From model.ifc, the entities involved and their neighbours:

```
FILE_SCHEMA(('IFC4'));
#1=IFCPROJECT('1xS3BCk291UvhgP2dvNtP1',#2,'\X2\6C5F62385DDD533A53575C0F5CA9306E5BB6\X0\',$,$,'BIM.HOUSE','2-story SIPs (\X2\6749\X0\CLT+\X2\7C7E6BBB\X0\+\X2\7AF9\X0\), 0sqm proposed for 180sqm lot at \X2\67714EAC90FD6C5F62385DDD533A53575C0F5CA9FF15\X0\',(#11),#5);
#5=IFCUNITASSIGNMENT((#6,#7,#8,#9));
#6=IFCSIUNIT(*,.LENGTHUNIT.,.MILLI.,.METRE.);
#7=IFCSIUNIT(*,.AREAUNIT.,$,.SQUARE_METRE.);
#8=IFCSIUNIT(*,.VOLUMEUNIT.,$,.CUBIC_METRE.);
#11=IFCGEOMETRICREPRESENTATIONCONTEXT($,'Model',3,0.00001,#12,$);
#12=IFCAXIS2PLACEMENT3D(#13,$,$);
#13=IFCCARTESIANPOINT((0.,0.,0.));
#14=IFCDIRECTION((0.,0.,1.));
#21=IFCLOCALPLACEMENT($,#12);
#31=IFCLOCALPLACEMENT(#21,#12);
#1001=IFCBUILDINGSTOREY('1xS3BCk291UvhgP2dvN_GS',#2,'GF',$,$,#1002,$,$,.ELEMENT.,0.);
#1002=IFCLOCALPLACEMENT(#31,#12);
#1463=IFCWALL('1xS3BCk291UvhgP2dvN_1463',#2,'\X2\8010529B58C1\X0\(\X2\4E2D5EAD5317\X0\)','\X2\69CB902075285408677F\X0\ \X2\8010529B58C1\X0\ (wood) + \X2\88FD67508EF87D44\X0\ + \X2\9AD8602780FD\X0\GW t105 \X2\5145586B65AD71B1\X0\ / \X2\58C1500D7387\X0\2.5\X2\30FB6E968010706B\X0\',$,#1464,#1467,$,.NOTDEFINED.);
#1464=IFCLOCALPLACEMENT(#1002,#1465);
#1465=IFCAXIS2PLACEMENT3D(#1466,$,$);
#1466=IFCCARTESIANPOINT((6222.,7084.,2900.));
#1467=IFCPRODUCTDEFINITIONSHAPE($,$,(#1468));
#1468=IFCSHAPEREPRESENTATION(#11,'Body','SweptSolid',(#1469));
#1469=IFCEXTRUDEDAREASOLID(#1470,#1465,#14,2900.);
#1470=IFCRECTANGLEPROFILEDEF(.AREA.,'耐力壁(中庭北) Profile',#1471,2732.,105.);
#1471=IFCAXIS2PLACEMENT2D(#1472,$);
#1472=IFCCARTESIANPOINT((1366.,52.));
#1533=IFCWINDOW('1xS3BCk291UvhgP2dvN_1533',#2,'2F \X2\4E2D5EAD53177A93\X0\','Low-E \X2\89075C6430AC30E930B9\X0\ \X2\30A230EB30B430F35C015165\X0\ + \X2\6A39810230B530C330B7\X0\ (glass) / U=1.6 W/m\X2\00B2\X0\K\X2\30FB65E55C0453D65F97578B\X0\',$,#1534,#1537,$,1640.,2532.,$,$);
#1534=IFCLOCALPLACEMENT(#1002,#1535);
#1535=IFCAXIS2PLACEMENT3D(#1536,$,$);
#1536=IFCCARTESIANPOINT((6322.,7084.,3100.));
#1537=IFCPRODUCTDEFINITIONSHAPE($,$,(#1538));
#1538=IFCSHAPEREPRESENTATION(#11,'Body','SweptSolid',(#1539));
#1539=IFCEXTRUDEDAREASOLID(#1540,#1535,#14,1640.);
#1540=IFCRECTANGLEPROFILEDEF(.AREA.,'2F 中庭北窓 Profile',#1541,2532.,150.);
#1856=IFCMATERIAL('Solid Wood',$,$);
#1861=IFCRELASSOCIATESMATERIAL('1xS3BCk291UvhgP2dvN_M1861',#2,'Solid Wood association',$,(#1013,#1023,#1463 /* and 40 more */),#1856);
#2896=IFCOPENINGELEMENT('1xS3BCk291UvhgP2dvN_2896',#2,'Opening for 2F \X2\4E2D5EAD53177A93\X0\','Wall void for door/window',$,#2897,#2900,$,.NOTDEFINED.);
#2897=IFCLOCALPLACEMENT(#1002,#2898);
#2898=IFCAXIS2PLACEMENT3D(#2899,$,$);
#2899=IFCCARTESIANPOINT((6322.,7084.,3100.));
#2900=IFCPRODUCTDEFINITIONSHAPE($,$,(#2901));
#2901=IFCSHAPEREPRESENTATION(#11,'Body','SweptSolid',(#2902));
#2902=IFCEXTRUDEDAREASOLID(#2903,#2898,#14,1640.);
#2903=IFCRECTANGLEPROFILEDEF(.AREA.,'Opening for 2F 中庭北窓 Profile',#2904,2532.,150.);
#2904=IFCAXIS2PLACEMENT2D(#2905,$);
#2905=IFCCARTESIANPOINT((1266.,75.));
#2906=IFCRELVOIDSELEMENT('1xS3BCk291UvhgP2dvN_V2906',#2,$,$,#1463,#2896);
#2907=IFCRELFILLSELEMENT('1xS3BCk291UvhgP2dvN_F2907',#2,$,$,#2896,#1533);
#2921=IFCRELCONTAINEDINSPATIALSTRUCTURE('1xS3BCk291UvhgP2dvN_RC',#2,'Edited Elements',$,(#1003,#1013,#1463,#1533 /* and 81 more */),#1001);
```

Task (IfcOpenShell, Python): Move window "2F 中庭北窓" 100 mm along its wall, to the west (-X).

```python
import ifcopenshell
import ifcopenshell.api.geometry
import ifcopenshell.util.placement

model = ifcopenshell.open("model.ifc")

window = model.by_id(1533)
opening = window.FillsVoids[0].RelatingOpeningElement
wall = opening.VoidsElements[0].RelatingBuildingElement

wall_matrix = ifcopenshell.util.placement.get_local_placement(wall.ObjectPlacement)
shift = wall_matrix[:3, 0] * -100.0
before = ifcopenshell.util.placement.get_local_placement(window.ObjectPlacement)[:3, 3].copy()

# The window is not placed relative to its opening, so move both.
for product in (opening, window):
    matrix = ifcopenshell.util.placement.get_local_placement(product.ObjectPlacement)
    matrix[:3, 3] += shift
    ifcopenshell.api.geometry.edit_object_placement(model, product=product, matrix=matrix, is_si=False)

after = ifcopenshell.util.placement.get_local_placement(window.ObjectPlacement)[:3, 3]
print("window moved by", (after - before).round(3) + 0.0)

model.write("model_rev.ifc")
```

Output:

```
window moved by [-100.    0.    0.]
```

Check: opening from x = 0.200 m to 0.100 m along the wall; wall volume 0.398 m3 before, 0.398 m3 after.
